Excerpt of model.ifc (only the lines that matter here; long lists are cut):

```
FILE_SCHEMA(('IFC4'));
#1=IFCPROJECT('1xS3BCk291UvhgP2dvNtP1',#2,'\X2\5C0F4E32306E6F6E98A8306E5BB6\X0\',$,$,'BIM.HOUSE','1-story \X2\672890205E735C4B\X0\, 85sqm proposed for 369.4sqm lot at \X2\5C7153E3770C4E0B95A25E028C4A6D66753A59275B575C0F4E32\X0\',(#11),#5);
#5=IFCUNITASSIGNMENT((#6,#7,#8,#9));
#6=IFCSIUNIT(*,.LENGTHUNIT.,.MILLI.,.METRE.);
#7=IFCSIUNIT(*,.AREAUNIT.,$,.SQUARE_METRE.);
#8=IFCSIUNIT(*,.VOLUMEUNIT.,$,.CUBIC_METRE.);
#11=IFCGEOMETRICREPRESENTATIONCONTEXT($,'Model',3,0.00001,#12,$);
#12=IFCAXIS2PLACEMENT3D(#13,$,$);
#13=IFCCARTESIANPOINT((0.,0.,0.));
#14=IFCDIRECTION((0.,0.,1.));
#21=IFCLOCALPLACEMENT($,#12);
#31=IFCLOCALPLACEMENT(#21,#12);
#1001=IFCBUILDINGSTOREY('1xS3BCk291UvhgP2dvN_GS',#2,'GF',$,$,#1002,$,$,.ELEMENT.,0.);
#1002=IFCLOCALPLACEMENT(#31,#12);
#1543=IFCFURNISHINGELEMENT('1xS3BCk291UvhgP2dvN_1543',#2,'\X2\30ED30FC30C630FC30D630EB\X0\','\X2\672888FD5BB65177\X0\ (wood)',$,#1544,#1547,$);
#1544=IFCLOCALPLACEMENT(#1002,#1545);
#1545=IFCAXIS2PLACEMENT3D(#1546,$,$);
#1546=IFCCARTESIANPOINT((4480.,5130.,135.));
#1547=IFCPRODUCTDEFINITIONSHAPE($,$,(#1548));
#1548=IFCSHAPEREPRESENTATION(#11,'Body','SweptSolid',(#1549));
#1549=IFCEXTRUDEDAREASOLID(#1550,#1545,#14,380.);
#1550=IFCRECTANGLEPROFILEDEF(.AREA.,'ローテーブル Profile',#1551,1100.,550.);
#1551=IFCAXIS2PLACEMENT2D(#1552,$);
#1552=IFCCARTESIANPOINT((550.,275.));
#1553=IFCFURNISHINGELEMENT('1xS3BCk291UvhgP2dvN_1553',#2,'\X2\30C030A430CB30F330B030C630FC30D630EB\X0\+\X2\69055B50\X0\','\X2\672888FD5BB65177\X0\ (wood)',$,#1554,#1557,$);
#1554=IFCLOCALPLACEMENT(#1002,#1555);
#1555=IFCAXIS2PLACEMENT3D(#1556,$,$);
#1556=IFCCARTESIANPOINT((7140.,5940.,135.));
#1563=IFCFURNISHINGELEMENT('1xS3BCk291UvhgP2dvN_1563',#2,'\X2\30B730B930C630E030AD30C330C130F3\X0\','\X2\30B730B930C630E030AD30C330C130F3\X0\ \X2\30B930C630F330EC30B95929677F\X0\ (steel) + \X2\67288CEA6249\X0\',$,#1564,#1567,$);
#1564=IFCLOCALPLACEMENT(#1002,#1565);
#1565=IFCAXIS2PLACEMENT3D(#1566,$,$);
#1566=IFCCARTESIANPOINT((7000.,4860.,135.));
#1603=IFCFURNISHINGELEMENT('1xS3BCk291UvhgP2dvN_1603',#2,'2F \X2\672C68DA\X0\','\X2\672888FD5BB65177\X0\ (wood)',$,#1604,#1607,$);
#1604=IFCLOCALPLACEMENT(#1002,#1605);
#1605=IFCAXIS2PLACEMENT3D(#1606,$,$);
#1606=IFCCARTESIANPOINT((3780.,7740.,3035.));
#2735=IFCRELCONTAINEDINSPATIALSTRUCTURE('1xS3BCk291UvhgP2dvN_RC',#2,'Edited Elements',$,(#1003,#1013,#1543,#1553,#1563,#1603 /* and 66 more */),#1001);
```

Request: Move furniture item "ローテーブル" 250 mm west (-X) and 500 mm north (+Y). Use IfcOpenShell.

```python
import ifcopenshell
import ifcopenshell.api.geometry
import ifcopenshell.util.placement
import ifcopenshell.util.unit

model = ifcopenshell.open("model.ifc")
unit_scale = ifcopenshell.util.unit.calculate_unit_scale(model)

item = model.by_id(1543)
matrix = ifcopenshell.util.placement.get_local_placement(item.ObjectPlacement)
matrix[0, 3] -= 0.25 / unit_scale
matrix[1, 3] += 0.5 / unit_scale
ifcopenshell.api.geometry.edit_object_placement(model, product=item, matrix=matrix, is_si=False)

print(ifcopenshell.util.placement.get_local_placement(item.ObjectPlacement).round(3) + 0.0)

model.write("model-out.ifc")
```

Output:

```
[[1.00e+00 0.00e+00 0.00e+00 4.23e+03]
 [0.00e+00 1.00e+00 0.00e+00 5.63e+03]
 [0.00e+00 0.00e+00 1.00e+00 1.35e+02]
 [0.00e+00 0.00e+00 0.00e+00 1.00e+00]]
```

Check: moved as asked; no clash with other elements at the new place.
